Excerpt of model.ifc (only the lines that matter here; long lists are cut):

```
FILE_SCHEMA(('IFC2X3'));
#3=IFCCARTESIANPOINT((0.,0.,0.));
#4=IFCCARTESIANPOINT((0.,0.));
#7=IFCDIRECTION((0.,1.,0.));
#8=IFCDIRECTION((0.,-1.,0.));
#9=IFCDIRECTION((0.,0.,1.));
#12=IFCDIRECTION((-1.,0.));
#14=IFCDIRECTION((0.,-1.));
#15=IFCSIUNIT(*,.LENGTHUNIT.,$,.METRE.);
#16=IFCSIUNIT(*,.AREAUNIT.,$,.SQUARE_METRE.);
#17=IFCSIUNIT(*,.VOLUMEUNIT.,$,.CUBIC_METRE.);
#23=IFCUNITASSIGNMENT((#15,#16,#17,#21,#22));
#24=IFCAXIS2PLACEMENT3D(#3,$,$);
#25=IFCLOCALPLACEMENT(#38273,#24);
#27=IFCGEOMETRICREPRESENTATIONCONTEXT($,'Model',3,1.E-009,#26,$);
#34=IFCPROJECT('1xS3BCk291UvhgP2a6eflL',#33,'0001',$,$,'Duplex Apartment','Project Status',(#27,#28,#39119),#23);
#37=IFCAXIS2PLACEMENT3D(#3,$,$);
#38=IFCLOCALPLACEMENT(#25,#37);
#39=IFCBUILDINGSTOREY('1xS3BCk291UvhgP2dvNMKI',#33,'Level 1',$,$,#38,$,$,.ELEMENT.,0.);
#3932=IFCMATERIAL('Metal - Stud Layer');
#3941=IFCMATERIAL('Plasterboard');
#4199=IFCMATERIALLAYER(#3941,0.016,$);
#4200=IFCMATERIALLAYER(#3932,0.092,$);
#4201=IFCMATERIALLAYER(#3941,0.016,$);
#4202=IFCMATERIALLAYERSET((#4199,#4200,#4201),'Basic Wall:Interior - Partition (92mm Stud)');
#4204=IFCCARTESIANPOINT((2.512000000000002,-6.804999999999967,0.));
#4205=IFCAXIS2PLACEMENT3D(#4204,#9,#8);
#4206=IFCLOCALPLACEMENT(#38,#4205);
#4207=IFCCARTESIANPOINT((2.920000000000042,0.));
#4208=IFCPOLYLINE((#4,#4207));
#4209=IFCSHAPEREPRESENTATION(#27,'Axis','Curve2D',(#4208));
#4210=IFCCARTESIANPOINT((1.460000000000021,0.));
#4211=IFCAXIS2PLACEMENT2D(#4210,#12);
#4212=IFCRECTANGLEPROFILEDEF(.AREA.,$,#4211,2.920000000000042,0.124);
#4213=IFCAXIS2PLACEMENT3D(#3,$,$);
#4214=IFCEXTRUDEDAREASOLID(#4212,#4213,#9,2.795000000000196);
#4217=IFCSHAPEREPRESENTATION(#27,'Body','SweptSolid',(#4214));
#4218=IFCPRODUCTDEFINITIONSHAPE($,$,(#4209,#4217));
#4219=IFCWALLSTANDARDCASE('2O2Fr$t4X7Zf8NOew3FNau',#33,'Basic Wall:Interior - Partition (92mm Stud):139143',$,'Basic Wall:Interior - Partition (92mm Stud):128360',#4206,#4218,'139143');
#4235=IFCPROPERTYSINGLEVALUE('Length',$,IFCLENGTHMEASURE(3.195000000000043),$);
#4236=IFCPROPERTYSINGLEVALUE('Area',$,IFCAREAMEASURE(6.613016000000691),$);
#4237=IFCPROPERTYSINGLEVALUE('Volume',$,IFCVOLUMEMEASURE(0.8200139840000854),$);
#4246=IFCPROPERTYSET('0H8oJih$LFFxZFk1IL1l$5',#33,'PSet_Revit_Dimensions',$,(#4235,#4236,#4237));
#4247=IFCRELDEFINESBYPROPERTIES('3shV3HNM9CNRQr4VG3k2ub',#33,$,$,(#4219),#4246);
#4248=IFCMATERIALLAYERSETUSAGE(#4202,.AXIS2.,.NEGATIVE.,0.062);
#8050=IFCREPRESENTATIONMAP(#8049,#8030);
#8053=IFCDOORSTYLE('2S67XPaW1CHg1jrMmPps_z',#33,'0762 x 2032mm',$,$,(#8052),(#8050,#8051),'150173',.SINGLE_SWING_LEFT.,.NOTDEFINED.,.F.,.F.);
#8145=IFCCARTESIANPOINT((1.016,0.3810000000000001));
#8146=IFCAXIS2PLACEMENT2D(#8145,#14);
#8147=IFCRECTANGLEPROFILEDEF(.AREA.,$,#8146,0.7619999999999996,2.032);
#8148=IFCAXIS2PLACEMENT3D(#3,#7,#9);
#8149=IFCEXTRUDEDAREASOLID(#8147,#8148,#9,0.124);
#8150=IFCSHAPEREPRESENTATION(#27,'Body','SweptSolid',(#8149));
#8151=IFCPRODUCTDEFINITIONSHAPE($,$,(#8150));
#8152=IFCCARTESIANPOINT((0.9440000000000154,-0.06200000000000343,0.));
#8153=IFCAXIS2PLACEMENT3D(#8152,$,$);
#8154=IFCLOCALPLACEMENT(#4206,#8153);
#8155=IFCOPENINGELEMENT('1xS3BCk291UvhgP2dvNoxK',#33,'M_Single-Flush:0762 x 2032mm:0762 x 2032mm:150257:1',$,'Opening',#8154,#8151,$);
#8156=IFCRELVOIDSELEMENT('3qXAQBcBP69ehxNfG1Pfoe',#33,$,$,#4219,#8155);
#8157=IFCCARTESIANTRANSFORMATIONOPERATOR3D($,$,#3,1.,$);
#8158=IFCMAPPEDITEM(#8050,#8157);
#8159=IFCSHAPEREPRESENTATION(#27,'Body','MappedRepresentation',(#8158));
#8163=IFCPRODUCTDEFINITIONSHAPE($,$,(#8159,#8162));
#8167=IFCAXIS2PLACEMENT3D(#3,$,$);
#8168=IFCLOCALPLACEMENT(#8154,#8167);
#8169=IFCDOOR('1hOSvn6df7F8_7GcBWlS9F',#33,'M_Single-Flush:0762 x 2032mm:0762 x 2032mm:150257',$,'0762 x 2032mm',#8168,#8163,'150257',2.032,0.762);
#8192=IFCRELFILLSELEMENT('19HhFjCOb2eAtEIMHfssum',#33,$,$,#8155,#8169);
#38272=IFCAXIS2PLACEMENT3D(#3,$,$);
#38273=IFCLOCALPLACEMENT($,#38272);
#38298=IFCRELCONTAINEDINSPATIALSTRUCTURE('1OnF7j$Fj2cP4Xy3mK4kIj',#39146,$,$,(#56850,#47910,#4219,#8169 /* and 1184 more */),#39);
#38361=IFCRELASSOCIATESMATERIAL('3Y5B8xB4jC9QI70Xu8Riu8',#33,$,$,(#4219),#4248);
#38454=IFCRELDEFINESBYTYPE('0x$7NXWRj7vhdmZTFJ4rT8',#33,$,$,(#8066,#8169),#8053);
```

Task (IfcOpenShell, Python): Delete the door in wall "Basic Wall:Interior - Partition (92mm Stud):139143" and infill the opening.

```python
import ifcopenshell
import ifcopenshell.api.feature
import ifcopenshell.api.pset
import ifcopenshell.api.root
import ifcopenshell.geom
import ifcopenshell.util.element
import ifcopenshell.util.shape
import ifcopenshell.util.unit

model = ifcopenshell.open("model.ifc")
area_scale = ifcopenshell.util.unit.calculate_unit_scale(model, "AREAUNIT")
volume_scale = ifcopenshell.util.unit.calculate_unit_scale(model, "VOLUMEUNIT")
settings = ifcopenshell.geom.settings()


def volume(element):
    """Net volume in cubic metres, openings subtracted."""
    shape = ifcopenshell.geom.create_shape(settings, element)
    return ifcopenshell.util.shape.get_volume(shape.geometry)


door = model.by_guid("1hOSvn6df7F8_7GcBWlS9F")
opening = door.FillsVoids[0].RelatingOpeningElement
wall = opening.VoidsElements[0].RelatingBuildingElement
before = volume(wall)

ifcopenshell.api.root.remove_product(model, product=door)
ifcopenshell.api.feature.remove_feature(model, feature=opening)

after = volume(wall)
thickness = 0.124  # wall thickness in metres

# Update the wall's stored quantities.
pset = model.by_id(ifcopenshell.util.element.get_pset(wall, "PSet_Revit_Dimensions", should_inherit=False)["id"])
ifcopenshell.api.pset.edit_pset(model, pset=pset, properties={
    "Area": model.create_entity("IfcAreaMeasure", after / thickness / area_scale),
    "Volume": model.create_entity("IfcVolumeMeasure", after / volume_scale),
})

print(f"wall volume {before:.3f} -> {after:.3f} m3")

model.write("model_edited.ifc")
```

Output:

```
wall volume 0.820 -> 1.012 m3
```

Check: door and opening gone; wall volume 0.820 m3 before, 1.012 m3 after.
